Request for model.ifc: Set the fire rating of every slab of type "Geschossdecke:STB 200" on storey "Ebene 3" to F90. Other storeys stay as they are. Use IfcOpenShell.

First a look at what the model holds.

```python
import ifcopenshell
import ifcopenshell.util.element

model = ifcopenshell.open("model.ifc")
print(model.schema)
storey = next(s for s in model.by_type("IfcBuildingStorey") if s.Name == "Ebene 3")
slabs = [e for e in ifcopenshell.util.element.get_decomposition(storey) if e.is_a("IfcSlab")]
seen = {}
for e in slabs:
    element_type = ifcopenshell.util.element.get_type(e)
    key = (element_type.Name if element_type != e and element_type else None, ifcopenshell.util.element.get_pset(e, "Pset_SlabCommon", "FireRating"))
    seen[key] = seen.get(key, 0) + 1
for (name, value), count in sorted(seen.items(), key=str):
    print(count, "x", name, "|", value)
```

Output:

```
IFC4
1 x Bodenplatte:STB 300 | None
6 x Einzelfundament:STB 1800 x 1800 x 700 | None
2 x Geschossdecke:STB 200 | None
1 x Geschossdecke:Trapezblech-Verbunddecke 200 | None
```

```python
import ifcopenshell
import ifcopenshell.api.pset
import ifcopenshell.util.element

model = ifcopenshell.open("model.ifc")

storey = next(s for s in model.by_type("IfcBuildingStorey") if s.Name == "Ebene 3")
slabs = [e for e in ifcopenshell.util.element.get_decomposition(storey) if e.is_a("IfcSlab")]

count = 0
for e in slabs:
    element_type = ifcopenshell.util.element.get_type(e)
    if element_type in (None, e) or element_type.Name != "Geschossdecke:STB 200":
        continue
    # add_pset returns the element's existing set when there is one.
    pset = ifcopenshell.api.pset.add_pset(model, product=e, name="Pset_SlabCommon")
    ifcopenshell.api.pset.edit_pset(model, pset=pset, properties={"FireRating": "F90"})
    count += 1

print(count, "slabs updated")

model.write("model_updated.ifc")
```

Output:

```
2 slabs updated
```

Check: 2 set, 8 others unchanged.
